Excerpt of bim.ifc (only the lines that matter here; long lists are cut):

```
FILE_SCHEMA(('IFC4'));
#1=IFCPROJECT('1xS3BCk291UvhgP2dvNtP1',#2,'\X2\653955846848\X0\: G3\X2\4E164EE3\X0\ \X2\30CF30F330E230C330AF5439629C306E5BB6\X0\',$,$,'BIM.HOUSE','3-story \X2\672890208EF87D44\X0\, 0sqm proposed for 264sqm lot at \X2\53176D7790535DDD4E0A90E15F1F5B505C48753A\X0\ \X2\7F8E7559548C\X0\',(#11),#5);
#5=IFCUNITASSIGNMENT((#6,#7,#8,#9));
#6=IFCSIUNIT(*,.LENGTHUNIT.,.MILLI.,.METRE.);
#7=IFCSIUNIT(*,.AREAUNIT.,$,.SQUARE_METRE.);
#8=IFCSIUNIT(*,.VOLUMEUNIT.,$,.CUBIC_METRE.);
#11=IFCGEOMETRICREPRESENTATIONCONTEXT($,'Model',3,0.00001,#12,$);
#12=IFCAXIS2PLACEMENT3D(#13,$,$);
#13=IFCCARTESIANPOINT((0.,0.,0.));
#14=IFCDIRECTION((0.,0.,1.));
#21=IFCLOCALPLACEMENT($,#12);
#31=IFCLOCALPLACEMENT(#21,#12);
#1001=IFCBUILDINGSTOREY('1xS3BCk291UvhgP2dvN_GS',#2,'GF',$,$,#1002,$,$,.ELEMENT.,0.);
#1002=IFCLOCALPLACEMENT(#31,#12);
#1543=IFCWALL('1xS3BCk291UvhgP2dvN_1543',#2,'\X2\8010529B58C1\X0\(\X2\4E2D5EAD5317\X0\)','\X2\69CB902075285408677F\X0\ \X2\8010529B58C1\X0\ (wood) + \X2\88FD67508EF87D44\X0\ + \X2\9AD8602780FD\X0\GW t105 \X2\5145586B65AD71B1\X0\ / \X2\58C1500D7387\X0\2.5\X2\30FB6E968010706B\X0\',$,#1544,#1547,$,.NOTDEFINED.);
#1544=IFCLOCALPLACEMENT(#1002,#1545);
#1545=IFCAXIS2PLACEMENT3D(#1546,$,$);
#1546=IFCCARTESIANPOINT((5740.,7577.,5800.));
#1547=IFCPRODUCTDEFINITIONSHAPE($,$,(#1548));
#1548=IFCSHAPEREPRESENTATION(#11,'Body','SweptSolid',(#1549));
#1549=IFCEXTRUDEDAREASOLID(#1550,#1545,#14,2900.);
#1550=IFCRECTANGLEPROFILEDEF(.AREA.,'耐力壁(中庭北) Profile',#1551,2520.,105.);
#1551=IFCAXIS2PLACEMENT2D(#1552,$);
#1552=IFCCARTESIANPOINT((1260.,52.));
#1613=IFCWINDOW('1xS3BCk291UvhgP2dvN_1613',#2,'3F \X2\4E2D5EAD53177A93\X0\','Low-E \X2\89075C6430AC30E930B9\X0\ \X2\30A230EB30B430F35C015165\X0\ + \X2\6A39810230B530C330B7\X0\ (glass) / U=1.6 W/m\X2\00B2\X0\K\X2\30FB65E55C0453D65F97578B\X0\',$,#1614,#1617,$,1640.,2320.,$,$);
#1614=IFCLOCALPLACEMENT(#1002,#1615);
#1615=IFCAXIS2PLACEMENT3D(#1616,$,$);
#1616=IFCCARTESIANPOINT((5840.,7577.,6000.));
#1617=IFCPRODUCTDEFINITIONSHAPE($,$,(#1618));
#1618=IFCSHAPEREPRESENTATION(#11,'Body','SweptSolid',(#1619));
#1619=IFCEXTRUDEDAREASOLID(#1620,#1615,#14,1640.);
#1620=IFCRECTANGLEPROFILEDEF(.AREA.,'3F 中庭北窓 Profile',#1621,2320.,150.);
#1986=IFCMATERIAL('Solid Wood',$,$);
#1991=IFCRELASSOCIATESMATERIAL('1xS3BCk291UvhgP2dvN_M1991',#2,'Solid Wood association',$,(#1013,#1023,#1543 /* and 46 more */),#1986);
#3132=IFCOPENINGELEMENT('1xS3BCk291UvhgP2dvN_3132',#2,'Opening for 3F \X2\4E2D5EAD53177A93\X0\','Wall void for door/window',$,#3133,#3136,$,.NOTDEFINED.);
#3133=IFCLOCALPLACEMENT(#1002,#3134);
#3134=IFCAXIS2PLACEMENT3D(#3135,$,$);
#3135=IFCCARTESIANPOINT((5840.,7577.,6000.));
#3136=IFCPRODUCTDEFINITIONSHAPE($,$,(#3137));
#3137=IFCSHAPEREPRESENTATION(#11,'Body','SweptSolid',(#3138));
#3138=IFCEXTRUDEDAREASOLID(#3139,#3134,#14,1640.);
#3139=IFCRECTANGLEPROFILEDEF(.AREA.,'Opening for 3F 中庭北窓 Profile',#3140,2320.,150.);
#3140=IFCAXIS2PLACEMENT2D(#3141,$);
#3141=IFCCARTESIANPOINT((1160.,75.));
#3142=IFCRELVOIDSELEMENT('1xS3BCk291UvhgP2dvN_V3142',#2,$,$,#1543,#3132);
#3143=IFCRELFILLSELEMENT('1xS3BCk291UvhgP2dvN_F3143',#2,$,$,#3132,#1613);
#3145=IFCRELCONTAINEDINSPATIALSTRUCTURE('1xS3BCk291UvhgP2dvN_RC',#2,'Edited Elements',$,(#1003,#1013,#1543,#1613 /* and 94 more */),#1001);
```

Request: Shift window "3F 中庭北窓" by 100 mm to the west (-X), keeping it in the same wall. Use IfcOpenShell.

```python
import ifcopenshell
import ifcopenshell.api.geometry
import ifcopenshell.util.placement

model = ifcopenshell.open("bim.ifc")

window = model.by_id(1613)
opening = window.FillsVoids[0].RelatingOpeningElement
wall = opening.VoidsElements[0].RelatingBuildingElement

wall_matrix = ifcopenshell.util.placement.get_local_placement(wall.ObjectPlacement)
shift = wall_matrix[:3, 0] * -100.0
before = ifcopenshell.util.placement.get_local_placement(window.ObjectPlacement)[:3, 3].copy()

# The window is not placed relative to its opening, so move both.
for product in (opening, window):
    matrix = ifcopenshell.util.placement.get_local_placement(product.ObjectPlacement)
    matrix[:3, 3] += shift
    ifcopenshell.api.geometry.edit_object_placement(model, product=product, matrix=matrix, is_si=False)

after = ifcopenshell.util.placement.get_local_placement(window.ObjectPlacement)[:3, 3]
print("window moved by", (after - before).round(3) + 0.0)

model.write("bim-out.ifc")
```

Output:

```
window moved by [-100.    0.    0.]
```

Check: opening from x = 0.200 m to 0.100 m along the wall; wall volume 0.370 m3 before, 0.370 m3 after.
